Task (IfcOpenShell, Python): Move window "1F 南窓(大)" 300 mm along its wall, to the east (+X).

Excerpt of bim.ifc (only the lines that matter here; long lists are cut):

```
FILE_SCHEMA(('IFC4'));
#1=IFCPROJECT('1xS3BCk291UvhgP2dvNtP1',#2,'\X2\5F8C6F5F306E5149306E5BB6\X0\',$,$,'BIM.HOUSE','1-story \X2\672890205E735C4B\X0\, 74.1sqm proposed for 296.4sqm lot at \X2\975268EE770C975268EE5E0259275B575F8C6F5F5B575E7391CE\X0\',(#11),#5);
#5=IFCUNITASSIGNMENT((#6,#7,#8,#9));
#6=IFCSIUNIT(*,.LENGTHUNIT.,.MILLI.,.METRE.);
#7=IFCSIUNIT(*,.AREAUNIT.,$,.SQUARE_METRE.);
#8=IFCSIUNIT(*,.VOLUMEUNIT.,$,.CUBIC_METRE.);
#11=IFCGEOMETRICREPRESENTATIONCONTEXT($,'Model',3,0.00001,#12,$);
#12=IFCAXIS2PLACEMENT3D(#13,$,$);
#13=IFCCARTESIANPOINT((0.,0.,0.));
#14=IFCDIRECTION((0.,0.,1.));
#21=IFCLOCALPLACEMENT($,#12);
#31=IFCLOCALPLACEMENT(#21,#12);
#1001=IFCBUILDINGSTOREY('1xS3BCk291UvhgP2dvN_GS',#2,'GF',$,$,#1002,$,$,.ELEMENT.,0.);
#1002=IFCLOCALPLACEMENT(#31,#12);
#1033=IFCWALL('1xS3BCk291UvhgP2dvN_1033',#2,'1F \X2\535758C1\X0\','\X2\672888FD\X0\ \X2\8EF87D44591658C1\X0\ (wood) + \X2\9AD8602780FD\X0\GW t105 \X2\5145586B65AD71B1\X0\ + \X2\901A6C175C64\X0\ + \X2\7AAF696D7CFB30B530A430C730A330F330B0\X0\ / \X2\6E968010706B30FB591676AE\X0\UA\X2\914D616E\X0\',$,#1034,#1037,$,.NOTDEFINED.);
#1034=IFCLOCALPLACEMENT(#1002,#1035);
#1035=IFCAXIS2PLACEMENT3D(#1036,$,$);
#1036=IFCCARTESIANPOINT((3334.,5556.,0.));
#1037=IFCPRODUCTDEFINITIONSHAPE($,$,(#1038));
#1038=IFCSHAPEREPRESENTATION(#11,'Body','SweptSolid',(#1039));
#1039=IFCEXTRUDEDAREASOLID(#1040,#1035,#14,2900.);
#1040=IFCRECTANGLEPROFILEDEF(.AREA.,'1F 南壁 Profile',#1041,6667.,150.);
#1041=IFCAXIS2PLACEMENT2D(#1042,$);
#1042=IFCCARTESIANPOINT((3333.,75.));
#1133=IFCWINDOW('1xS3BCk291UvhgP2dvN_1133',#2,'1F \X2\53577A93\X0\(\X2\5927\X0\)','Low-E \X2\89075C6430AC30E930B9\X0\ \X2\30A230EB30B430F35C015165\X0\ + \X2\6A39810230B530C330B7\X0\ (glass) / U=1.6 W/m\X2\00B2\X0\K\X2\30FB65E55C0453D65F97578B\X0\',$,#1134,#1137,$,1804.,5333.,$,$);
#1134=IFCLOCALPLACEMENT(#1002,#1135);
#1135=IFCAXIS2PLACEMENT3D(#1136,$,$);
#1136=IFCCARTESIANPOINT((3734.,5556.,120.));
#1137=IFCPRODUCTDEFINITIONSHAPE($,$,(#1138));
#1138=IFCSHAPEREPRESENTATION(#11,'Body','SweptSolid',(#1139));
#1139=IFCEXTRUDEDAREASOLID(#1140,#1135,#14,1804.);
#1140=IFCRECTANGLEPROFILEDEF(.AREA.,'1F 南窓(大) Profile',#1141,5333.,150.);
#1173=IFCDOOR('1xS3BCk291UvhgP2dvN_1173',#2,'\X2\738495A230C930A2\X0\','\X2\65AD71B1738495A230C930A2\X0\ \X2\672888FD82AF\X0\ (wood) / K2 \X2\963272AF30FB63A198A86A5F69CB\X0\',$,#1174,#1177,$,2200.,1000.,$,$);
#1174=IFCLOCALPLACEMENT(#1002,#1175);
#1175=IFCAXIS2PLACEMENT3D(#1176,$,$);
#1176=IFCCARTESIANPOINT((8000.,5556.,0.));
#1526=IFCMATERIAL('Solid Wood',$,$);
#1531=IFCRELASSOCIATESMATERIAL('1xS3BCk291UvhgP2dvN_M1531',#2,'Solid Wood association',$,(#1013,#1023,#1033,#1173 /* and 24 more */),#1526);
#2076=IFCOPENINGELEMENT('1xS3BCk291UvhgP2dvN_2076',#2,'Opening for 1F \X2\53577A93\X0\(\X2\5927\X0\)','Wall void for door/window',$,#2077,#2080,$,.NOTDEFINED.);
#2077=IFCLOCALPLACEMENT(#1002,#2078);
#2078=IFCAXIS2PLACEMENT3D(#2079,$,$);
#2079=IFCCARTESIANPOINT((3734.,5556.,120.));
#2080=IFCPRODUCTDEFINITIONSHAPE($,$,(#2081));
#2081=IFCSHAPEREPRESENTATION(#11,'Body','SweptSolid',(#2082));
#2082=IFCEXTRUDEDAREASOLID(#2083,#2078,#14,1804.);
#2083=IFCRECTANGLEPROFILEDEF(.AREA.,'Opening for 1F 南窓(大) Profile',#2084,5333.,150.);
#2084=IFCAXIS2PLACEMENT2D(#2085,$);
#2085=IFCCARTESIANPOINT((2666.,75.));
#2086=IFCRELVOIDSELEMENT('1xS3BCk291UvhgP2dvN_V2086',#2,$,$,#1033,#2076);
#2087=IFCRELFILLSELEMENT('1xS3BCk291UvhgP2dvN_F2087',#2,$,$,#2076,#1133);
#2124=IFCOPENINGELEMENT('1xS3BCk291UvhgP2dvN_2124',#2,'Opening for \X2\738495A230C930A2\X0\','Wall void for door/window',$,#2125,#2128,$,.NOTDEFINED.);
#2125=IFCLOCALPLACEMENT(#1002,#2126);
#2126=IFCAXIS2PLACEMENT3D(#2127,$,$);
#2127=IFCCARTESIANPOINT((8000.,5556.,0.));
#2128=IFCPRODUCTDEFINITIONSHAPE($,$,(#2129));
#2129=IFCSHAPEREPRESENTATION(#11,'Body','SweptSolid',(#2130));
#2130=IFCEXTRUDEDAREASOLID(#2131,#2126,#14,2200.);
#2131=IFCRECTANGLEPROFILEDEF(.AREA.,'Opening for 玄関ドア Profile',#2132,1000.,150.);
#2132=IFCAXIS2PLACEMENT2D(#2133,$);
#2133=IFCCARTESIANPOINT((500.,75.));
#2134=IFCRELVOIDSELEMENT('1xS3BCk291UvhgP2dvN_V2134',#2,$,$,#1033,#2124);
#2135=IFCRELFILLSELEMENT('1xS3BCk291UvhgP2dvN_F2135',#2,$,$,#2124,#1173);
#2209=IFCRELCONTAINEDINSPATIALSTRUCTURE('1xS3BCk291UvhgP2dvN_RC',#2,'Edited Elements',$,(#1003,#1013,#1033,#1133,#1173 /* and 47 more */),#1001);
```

```python
import ifcopenshell
import ifcopenshell.api.geometry
import ifcopenshell.util.placement
import ifcopenshell.util.unit

model = ifcopenshell.open("bim.ifc")
unit_scale = ifcopenshell.util.unit.calculate_unit_scale(model)

window = model.by_guid("1xS3BCk291UvhgP2dvN_1133")
opening = window.FillsVoids[0].RelatingOpeningElement
wall = opening.VoidsElements[0].RelatingBuildingElement

wall_matrix = ifcopenshell.util.placement.get_local_placement(wall.ObjectPlacement)
shift = wall_matrix[:3, 0] * 0.3 / unit_scale
before = ifcopenshell.util.placement.get_local_placement(window.ObjectPlacement)[:3, 3].copy()

# The window is not placed relative to its opening, so move both.
for product in (opening, window):
    matrix = ifcopenshell.util.placement.get_local_placement(product.ObjectPlacement)
    matrix[:3, 3] += shift
    ifcopenshell.api.geometry.edit_object_placement(model, product=product, matrix=matrix, is_si=False)

after = ifcopenshell.util.placement.get_local_placement(window.ObjectPlacement)[:3, 3]
print("window moved by", (after - before).round(3) + 0.0)

model.write("bim_rev.ifc")
```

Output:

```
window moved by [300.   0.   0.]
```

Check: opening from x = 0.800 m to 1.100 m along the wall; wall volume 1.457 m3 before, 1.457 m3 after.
